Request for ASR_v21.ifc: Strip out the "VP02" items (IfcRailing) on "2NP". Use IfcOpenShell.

First a look at what the model holds.

```python
import ifcopenshell
import ifcopenshell.util.element

model = ifcopenshell.open("ASR_v21.ifc")
print(model.schema)
storey = next(s for s in model.by_type("IfcBuildingStorey") if s.Name == "2NP")
railings = [e for e in ifcopenshell.util.element.get_decomposition(storey) if e.is_a("IfcRailing")]
seen = {}
for e in railings:
    element_type = ifcopenshell.util.element.get_type(e)
    name = element_type.Name if element_type not in (None, e) else None
    seen[name] = seen.get(name, 0) + 1
for name, count in sorted(seen.items(), key=str):
    print(count, "x", name)
```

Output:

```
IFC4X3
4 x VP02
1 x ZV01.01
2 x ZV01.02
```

```python
import ifcopenshell
import ifcopenshell.api.root
import ifcopenshell.util.element

model = ifcopenshell.open("ASR_v21.ifc")

storey = next(s for s in model.by_type("IfcBuildingStorey") if s.Name == "2NP")
railings = [e for e in ifcopenshell.util.element.get_decomposition(storey) if e.is_a("IfcRailing")]
targets = [e for e in railings if (t := ifcopenshell.util.element.get_type(e)) not in (None, e) and t.Name == "VP02"]

for e in targets:
    ifcopenshell.api.root.remove_product(model, product=e)
print(len(targets), "removed")

model.write("ASR_v21_v2.ifc")
```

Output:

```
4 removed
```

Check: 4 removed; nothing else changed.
